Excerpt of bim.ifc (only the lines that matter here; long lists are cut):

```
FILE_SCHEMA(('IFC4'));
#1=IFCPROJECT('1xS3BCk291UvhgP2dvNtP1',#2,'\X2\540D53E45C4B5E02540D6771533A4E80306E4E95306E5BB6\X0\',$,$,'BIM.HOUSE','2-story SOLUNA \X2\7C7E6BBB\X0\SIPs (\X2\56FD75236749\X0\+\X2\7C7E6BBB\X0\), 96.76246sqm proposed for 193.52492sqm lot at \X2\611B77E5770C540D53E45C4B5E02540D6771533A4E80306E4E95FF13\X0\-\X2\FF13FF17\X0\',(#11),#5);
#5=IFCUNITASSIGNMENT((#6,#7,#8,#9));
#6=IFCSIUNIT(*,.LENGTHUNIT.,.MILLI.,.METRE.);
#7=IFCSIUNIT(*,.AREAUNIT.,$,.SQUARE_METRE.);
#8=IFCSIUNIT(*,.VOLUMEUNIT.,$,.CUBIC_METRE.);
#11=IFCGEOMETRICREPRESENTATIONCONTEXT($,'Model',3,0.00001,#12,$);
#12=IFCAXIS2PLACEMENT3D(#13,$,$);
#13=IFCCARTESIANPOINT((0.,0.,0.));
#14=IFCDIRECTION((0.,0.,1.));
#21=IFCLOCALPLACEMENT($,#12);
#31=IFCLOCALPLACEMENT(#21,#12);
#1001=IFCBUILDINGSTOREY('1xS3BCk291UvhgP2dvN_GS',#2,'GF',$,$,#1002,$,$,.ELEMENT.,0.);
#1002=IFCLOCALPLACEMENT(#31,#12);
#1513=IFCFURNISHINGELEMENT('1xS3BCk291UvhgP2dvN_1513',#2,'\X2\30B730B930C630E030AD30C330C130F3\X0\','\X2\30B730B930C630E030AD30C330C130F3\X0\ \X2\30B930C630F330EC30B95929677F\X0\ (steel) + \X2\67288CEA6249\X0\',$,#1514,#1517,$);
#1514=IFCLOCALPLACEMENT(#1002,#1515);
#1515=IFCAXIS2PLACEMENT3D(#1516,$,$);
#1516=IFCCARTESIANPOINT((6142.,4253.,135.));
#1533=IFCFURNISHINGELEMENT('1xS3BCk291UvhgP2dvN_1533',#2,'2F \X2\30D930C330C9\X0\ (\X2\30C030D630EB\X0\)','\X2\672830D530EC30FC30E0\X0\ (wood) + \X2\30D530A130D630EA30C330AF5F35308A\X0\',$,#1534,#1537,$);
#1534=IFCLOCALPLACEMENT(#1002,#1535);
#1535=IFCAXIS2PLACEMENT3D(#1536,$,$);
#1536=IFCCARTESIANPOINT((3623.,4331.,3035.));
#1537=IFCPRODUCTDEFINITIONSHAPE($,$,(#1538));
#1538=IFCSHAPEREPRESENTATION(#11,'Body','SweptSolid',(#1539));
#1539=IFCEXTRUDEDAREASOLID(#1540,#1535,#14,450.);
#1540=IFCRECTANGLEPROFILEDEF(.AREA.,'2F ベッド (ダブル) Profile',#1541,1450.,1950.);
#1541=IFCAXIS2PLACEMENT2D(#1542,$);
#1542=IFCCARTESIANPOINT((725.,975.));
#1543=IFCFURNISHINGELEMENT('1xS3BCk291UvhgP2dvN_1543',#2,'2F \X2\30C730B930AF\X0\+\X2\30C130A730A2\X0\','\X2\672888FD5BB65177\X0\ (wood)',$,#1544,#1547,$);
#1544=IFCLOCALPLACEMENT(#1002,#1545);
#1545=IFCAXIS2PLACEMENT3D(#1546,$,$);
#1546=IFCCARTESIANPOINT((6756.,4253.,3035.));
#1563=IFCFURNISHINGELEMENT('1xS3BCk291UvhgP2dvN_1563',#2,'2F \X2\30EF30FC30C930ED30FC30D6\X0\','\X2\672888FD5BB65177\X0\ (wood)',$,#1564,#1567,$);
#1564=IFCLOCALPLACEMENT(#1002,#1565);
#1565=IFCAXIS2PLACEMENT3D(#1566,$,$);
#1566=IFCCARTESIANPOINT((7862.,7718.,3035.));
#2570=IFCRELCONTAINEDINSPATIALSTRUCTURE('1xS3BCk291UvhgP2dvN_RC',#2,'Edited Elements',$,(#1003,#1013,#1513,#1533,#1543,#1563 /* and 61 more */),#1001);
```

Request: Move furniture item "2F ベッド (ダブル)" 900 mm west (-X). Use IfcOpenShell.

```python
import ifcopenshell
import ifcopenshell.api.geometry
import ifcopenshell.util.placement

model = ifcopenshell.open("bim.ifc")

item = model.by_guid("1xS3BCk291UvhgP2dvN_1533")
matrix = ifcopenshell.util.placement.get_local_placement(item.ObjectPlacement)
matrix[0, 3] -= 900.0
ifcopenshell.api.geometry.edit_object_placement(model, product=item, matrix=matrix, is_si=False)

print(ifcopenshell.util.placement.get_local_placement(item.ObjectPlacement).round(3) + 0.0)

model.write("bim_rev.ifc")
```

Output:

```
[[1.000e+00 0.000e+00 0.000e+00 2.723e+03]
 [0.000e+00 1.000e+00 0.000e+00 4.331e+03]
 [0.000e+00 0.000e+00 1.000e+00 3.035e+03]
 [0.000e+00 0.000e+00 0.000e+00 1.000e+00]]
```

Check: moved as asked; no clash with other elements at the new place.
